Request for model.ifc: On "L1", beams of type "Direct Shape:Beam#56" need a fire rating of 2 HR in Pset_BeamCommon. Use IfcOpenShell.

First a look at what the model holds.

```python
import ifcopenshell
import ifcopenshell.util.element

model = ifcopenshell.open("model.ifc")
print(model.schema)
storey = next(s for s in model.by_type("IfcBuildingStorey") if s.Name == "L1")
beams = [e for e in ifcopenshell.util.element.get_decomposition(storey) if e.is_a("IfcBeam")]
seen = {}
for e in beams:
    element_type = ifcopenshell.util.element.get_type(e)
    key = (element_type.Name if element_type != e and element_type else None, ifcopenshell.util.element.get_pset(e, "Pset_BeamCommon", "FireRating"))
    seen[key] = seen.get(key, 0) + 1
for (name, value), count in sorted(seen.items(), key=str):
    print(count, "x", name, "|", value)
```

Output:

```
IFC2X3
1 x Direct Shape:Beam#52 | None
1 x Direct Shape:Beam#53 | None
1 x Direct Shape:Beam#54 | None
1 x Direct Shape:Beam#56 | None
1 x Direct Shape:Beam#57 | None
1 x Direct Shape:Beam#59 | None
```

```python
import ifcopenshell
import ifcopenshell.api.pset
import ifcopenshell.util.element

model = ifcopenshell.open("model.ifc")

storey = next(s for s in model.by_type("IfcBuildingStorey") if s.Name == "L1")
beams = [e for e in ifcopenshell.util.element.get_decomposition(storey) if e.is_a("IfcBeam")]

count = 0
for e in beams:
    element_type = ifcopenshell.util.element.get_type(e)
    if element_type in (None, e) or element_type.Name != "Direct Shape:Beam#56":
        continue
    # add_pset returns the element's existing set when there is one.
    pset = ifcopenshell.api.pset.add_pset(model, product=e, name="Pset_BeamCommon")
    ifcopenshell.api.pset.edit_pset(model, pset=pset, properties={"FireRating": "2 HR"})
    count += 1

print(count, "beams updated")

model.write("model_edited.ifc")
```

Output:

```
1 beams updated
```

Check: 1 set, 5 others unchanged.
